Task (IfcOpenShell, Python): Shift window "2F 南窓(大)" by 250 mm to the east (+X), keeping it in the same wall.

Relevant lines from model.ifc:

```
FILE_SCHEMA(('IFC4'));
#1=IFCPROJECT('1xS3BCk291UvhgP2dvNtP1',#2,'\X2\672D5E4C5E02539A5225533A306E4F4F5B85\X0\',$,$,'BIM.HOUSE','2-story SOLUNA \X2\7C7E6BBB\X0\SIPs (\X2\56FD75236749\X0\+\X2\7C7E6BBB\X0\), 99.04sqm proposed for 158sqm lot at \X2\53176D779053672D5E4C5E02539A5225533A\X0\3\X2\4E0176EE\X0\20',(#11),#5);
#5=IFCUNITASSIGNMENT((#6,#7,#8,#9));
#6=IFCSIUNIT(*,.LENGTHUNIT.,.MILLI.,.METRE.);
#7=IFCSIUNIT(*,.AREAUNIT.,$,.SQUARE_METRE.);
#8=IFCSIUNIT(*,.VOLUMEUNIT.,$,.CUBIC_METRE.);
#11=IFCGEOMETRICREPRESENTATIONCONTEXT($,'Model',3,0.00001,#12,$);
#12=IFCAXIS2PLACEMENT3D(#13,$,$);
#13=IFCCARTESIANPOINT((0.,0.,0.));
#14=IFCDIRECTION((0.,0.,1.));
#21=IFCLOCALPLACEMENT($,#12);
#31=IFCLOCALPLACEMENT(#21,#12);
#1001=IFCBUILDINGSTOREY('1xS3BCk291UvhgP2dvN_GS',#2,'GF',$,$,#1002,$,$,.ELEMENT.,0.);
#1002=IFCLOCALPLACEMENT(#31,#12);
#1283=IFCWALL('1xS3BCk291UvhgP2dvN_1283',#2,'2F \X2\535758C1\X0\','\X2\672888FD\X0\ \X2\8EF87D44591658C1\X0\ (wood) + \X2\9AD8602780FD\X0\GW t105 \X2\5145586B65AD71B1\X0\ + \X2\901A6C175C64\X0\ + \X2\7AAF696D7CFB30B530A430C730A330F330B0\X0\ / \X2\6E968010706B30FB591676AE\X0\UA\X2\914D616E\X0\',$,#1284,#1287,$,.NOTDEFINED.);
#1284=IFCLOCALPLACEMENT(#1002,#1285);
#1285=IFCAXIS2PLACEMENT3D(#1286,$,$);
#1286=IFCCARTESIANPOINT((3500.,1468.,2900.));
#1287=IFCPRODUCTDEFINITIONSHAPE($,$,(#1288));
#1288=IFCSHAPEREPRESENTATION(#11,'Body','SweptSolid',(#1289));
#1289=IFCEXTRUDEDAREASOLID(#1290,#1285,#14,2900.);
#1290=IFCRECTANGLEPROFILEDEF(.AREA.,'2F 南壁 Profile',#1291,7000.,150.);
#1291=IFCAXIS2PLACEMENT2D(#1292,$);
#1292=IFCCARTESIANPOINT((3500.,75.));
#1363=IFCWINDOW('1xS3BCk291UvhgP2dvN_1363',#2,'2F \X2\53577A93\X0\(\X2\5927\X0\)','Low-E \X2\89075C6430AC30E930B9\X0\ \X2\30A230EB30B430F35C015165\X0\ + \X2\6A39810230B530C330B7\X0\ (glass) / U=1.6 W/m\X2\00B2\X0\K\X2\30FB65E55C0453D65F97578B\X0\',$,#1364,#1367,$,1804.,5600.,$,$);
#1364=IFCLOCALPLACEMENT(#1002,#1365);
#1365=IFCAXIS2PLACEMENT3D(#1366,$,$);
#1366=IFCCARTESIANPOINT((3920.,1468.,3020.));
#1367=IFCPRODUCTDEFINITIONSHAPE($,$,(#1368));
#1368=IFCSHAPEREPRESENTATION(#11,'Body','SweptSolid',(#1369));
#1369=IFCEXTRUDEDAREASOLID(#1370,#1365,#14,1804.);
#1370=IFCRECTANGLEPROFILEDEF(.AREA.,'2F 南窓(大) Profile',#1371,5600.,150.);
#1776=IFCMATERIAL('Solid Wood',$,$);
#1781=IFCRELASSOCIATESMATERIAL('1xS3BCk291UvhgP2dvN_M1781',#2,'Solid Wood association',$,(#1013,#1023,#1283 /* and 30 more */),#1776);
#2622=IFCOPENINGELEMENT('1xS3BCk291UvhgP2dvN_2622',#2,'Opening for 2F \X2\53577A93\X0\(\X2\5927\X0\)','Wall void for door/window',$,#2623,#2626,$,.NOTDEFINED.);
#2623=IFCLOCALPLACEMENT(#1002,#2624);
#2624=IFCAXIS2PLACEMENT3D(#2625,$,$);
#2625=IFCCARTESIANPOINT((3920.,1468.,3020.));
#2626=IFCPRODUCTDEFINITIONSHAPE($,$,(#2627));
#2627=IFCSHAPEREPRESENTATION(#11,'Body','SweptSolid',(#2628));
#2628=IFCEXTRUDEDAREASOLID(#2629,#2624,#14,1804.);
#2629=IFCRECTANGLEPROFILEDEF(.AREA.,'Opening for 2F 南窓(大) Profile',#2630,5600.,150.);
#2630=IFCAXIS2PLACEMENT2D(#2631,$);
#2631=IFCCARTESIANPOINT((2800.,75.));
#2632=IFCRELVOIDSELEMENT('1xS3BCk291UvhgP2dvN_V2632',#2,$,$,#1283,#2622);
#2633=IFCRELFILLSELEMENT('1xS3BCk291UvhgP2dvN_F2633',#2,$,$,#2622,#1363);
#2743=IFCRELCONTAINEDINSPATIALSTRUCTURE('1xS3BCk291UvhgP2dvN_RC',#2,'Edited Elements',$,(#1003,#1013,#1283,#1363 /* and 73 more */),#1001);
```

```python
import ifcopenshell
import ifcopenshell.api.geometry
import ifcopenshell.util.placement

model = ifcopenshell.open("model.ifc")

window = model.by_guid("1xS3BCk291UvhgP2dvN_1363")
opening = window.FillsVoids[0].RelatingOpeningElement
wall = opening.VoidsElements[0].RelatingBuildingElement

wall_matrix = ifcopenshell.util.placement.get_local_placement(wall.ObjectPlacement)
shift = wall_matrix[:3, 0] * 250.0
before = ifcopenshell.util.placement.get_local_placement(window.ObjectPlacement)[:3, 3].copy()

# The window is not placed relative to its opening, so move both.
for product in (opening, window):
    matrix = ifcopenshell.util.placement.get_local_placement(product.ObjectPlacement)
    matrix[:3, 3] += shift
    ifcopenshell.api.geometry.edit_object_placement(model, product=product, matrix=matrix, is_si=False)

after = ifcopenshell.util.placement.get_local_placement(window.ObjectPlacement)[:3, 3]
print("window moved by", (after - before).round(3) + 0.0)

model.write("model_v2.ifc")
```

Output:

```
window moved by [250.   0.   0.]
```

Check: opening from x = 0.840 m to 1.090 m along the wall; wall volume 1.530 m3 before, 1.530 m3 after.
